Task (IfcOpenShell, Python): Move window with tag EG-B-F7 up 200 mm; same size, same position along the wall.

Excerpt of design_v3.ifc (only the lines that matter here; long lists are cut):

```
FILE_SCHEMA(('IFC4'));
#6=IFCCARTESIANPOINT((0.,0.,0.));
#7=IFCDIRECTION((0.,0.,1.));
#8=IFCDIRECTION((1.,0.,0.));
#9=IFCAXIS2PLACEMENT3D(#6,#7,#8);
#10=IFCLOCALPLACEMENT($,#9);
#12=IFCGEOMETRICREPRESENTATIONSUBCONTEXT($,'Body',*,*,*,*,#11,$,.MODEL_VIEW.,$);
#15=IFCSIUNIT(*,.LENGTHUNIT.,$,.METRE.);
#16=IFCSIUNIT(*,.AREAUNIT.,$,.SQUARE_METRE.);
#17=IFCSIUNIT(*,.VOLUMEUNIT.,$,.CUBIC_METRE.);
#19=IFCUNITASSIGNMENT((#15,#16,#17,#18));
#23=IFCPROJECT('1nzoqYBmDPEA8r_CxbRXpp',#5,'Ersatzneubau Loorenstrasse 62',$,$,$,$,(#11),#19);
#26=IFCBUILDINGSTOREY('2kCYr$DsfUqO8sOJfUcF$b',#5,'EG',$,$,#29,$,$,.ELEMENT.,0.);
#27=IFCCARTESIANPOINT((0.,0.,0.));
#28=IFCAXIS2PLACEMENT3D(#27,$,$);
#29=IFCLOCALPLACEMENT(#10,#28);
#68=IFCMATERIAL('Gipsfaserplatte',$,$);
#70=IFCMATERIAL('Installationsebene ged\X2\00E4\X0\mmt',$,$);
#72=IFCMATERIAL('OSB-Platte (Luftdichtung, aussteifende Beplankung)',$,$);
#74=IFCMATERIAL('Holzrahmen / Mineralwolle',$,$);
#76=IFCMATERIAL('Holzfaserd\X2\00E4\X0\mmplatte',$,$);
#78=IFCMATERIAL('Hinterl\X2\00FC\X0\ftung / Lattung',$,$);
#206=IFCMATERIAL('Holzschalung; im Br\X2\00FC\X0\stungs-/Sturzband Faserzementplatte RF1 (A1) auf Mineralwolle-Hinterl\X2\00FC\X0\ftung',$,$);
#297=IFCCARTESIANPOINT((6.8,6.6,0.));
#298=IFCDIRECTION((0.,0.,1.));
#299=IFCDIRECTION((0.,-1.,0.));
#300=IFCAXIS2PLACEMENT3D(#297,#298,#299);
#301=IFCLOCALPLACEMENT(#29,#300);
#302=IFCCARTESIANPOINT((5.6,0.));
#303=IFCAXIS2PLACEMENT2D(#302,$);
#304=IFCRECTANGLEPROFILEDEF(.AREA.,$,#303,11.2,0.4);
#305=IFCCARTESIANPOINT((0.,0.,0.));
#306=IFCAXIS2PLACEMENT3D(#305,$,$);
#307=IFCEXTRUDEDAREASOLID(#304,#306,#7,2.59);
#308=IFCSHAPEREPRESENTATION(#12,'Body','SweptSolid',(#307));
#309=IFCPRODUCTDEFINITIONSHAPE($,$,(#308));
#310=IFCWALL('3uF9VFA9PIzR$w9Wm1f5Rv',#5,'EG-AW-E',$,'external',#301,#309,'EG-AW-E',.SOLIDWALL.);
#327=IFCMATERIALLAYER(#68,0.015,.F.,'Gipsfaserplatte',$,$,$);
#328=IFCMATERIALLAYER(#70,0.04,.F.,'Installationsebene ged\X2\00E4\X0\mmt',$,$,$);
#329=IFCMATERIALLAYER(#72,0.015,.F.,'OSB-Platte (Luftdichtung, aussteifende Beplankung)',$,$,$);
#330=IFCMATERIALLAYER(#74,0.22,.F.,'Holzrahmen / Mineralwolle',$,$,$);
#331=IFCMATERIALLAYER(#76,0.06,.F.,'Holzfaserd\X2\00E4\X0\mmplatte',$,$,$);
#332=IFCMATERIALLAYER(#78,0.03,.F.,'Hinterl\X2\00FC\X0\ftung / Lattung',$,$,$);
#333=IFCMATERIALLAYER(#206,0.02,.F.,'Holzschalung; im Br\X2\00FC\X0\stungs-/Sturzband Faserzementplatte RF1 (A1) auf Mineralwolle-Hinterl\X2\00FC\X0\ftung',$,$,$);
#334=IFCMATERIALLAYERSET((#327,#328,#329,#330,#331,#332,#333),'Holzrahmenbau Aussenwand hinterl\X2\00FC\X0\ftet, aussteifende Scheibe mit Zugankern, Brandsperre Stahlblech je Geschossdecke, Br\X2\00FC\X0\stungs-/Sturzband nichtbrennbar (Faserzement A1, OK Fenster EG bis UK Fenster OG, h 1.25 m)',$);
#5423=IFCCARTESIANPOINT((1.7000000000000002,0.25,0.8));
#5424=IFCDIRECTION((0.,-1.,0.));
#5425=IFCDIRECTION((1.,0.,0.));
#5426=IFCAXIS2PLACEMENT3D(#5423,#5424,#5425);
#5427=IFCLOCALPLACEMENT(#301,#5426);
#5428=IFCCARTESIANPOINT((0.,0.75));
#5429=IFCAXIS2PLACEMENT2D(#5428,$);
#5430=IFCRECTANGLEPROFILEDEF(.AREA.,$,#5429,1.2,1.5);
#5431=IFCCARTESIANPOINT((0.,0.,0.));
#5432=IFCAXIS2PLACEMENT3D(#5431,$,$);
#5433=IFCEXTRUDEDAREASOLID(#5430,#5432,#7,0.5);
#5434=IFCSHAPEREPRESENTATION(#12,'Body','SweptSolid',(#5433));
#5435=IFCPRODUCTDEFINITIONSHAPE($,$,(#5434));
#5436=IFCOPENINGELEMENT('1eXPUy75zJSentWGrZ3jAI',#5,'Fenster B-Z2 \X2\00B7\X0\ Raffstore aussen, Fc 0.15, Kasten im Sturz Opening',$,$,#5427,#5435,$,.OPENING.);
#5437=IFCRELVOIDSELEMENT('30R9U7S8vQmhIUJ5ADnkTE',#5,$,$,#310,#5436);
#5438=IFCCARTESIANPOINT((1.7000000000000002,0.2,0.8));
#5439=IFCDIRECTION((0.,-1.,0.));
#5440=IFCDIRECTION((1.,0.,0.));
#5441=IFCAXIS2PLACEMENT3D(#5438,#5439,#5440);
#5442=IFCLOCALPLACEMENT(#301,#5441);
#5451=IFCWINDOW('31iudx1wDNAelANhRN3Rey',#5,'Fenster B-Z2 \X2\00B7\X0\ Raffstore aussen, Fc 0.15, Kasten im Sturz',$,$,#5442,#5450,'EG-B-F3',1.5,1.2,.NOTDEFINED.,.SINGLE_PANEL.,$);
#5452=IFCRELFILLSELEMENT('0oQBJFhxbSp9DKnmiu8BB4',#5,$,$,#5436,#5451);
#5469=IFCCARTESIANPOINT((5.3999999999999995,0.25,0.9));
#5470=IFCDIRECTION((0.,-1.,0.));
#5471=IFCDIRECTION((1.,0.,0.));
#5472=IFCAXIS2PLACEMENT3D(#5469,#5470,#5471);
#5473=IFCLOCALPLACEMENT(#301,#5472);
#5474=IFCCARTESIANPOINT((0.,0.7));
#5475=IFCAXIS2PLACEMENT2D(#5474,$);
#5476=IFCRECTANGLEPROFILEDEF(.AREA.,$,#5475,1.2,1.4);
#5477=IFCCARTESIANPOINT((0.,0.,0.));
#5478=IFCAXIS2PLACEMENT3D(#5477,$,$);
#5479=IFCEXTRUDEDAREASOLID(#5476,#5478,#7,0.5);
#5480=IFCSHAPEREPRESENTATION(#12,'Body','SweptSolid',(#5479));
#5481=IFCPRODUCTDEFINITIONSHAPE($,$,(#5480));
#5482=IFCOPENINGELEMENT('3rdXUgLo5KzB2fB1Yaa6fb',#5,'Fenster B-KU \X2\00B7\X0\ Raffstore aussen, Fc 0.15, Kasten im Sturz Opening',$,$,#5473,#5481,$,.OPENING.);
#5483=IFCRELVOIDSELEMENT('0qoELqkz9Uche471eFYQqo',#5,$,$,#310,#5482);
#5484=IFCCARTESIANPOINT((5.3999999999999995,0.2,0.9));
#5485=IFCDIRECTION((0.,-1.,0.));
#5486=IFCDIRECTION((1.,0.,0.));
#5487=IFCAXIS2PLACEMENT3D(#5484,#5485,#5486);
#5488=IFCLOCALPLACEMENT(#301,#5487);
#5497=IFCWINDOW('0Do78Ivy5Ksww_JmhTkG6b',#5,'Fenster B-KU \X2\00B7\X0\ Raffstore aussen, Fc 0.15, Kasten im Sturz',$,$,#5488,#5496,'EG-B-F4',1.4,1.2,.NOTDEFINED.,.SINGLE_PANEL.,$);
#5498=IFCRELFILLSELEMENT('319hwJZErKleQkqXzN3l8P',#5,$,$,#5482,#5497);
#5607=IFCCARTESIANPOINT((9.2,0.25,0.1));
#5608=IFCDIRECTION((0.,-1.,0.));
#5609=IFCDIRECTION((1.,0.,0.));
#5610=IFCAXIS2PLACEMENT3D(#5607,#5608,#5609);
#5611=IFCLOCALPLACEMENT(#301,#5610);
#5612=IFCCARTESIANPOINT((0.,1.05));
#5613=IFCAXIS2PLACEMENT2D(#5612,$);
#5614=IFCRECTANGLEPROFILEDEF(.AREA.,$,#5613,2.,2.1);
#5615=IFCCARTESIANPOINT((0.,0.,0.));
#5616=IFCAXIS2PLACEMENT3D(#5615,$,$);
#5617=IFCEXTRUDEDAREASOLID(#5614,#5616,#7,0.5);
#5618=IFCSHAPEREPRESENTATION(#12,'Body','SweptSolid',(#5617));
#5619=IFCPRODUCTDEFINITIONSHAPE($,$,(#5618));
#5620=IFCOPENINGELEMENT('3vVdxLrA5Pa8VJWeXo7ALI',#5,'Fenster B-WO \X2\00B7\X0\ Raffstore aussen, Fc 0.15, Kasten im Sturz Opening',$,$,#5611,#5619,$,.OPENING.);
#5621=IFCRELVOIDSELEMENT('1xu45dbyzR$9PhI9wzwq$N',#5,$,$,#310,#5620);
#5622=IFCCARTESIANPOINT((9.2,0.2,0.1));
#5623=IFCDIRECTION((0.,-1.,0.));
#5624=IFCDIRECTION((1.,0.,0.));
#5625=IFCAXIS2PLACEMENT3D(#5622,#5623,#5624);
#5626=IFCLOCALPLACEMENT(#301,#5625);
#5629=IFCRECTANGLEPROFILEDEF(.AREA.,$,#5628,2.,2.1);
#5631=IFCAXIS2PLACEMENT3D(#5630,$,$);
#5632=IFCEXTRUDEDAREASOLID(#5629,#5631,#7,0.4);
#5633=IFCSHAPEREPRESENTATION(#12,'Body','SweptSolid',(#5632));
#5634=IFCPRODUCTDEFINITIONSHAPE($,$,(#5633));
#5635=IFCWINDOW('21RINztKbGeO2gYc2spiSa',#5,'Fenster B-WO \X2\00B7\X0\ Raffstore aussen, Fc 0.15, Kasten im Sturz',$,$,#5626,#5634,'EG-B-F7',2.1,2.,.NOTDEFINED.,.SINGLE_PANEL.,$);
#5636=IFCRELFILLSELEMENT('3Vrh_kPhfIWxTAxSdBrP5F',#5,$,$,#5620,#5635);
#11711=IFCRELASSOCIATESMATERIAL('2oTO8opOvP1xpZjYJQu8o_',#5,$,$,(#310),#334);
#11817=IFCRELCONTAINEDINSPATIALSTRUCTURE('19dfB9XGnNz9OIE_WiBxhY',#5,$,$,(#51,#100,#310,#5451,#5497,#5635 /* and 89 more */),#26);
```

```python
import numpy as np
import ifcopenshell
import ifcopenshell.api.geometry
import ifcopenshell.util.placement
import ifcopenshell.util.unit

model = ifcopenshell.open("design_v3.ifc")
unit_scale = ifcopenshell.util.unit.calculate_unit_scale(model)

window = model.by_guid("21RINztKbGeO2gYc2spiSa")
opening = window.FillsVoids[0].RelatingOpeningElement
dz = 0.2 / unit_scale

shift = np.array([0.0, 0.0, dz])
# The window is not placed relative to its opening, so move both.
for product in (opening, window):
    matrix = ifcopenshell.util.placement.get_local_placement(product.ObjectPlacement)
    matrix[:3, 3] += shift
    ifcopenshell.api.geometry.edit_object_placement(model, product=product, matrix=matrix, is_si=False)

print(f"moved by {dz * unit_scale:+.3f} m")

model.write("design_v3_updated.ifc")
```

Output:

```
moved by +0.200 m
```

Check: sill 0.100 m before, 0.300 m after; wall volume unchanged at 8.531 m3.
